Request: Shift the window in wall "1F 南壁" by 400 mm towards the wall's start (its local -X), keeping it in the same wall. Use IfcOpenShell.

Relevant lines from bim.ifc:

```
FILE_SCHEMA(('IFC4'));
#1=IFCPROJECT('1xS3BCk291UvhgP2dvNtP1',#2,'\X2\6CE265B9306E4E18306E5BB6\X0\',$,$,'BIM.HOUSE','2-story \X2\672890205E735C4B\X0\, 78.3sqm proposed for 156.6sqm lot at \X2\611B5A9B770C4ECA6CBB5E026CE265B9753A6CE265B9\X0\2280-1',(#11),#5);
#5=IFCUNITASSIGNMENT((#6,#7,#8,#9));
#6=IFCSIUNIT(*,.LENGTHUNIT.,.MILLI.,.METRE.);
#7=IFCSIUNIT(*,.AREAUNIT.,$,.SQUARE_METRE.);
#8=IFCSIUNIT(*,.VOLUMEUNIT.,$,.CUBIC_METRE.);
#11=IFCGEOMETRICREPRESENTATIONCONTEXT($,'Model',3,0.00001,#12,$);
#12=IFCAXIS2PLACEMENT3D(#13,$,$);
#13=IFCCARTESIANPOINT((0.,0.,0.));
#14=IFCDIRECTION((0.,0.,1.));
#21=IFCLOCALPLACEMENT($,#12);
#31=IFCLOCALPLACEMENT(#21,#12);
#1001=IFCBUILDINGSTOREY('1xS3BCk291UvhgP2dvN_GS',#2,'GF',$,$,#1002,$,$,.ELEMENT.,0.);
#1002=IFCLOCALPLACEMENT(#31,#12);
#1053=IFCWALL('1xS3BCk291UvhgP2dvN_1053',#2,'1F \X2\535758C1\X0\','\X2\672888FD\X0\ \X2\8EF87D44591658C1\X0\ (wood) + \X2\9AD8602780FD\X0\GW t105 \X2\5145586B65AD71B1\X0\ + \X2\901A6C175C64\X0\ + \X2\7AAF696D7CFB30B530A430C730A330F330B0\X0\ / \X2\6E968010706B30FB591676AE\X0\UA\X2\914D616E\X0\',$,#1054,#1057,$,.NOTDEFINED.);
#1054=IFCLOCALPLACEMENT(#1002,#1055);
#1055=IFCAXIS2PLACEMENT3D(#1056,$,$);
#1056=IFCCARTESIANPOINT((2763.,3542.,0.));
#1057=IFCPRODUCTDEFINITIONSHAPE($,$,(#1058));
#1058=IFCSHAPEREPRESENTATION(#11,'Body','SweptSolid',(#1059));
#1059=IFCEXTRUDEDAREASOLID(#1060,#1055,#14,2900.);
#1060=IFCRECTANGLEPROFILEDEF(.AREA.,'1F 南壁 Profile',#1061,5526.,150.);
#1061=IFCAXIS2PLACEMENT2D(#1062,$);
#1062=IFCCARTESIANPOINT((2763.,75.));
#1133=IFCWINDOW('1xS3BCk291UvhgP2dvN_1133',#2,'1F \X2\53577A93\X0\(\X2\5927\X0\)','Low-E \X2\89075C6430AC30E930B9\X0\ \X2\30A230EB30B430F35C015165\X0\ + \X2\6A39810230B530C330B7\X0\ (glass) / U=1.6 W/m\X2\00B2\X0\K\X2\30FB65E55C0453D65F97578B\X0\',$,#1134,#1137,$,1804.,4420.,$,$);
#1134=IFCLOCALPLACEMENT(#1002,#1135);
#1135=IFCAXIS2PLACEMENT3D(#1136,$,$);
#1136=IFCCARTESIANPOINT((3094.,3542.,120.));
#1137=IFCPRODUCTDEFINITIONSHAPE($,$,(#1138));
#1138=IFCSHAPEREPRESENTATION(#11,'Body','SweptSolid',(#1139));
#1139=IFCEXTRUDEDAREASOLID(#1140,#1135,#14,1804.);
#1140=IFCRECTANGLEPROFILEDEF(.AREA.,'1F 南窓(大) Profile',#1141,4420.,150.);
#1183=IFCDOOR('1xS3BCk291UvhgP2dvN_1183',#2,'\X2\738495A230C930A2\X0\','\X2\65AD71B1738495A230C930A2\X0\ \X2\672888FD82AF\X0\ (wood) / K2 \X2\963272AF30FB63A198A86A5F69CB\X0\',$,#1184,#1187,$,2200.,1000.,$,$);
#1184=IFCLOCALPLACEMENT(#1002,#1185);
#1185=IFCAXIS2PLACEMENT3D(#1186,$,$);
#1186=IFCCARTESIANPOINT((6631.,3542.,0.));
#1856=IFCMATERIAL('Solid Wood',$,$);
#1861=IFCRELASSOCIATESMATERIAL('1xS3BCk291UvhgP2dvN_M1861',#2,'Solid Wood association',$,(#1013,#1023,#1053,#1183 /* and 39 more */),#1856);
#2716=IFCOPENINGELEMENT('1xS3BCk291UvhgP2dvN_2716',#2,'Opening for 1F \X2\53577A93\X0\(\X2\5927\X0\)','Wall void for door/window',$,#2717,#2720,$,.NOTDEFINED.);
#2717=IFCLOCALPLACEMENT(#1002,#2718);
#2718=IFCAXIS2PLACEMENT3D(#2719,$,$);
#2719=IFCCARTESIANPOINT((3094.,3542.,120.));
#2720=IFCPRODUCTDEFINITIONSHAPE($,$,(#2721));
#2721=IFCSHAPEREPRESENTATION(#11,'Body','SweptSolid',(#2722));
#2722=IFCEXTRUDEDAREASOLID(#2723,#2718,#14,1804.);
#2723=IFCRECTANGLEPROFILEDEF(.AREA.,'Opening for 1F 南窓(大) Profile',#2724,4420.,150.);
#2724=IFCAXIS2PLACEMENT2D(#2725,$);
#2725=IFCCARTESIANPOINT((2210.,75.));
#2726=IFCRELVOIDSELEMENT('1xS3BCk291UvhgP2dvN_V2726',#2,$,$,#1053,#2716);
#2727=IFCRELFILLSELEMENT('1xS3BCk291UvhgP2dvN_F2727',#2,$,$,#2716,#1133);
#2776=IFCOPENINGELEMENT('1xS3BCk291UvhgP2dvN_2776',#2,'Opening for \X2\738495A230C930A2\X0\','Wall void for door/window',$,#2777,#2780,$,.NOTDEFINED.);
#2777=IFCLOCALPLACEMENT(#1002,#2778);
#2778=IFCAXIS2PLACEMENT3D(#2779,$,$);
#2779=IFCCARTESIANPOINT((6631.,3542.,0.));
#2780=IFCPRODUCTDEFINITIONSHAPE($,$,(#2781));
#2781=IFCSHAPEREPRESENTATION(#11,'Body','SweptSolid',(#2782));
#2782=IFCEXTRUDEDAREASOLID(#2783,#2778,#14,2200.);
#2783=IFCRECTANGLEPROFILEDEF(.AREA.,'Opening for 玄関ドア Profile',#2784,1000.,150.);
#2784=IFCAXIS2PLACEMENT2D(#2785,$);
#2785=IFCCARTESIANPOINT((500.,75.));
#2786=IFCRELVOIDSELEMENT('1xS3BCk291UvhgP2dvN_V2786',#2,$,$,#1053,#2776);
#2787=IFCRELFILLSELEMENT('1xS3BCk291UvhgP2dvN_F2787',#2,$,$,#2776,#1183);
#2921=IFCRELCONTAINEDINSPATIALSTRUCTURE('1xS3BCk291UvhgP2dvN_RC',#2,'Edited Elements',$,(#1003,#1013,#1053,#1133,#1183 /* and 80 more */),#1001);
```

```python
import ifcopenshell
import ifcopenshell.api.geometry
import ifcopenshell.util.placement
import ifcopenshell.util.unit

model = ifcopenshell.open("bim.ifc")
unit_scale = ifcopenshell.util.unit.calculate_unit_scale(model)

window = model.by_guid("1xS3BCk291UvhgP2dvN_1133")
opening = window.FillsVoids[0].RelatingOpeningElement
wall = opening.VoidsElements[0].RelatingBuildingElement

wall_matrix = ifcopenshell.util.placement.get_local_placement(wall.ObjectPlacement)
shift = wall_matrix[:3, 0] * -0.4 / unit_scale
before = ifcopenshell.util.placement.get_local_placement(window.ObjectPlacement)[:3, 3].copy()

# The window is not placed relative to its opening, so move both.
for product in (opening, window):
    matrix = ifcopenshell.util.placement.get_local_placement(product.ObjectPlacement)
    matrix[:3, 3] += shift
    ifcopenshell.api.geometry.edit_object_placement(model, product=product, matrix=matrix, is_si=False)

after = ifcopenshell.util.placement.get_local_placement(window.ObjectPlacement)[:3, 3]
print("window moved by", (after - before).round(3) + 0.0)

model.write("bim-out.ifc")
```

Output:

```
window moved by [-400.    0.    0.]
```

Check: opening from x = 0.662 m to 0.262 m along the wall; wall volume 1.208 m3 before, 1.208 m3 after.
